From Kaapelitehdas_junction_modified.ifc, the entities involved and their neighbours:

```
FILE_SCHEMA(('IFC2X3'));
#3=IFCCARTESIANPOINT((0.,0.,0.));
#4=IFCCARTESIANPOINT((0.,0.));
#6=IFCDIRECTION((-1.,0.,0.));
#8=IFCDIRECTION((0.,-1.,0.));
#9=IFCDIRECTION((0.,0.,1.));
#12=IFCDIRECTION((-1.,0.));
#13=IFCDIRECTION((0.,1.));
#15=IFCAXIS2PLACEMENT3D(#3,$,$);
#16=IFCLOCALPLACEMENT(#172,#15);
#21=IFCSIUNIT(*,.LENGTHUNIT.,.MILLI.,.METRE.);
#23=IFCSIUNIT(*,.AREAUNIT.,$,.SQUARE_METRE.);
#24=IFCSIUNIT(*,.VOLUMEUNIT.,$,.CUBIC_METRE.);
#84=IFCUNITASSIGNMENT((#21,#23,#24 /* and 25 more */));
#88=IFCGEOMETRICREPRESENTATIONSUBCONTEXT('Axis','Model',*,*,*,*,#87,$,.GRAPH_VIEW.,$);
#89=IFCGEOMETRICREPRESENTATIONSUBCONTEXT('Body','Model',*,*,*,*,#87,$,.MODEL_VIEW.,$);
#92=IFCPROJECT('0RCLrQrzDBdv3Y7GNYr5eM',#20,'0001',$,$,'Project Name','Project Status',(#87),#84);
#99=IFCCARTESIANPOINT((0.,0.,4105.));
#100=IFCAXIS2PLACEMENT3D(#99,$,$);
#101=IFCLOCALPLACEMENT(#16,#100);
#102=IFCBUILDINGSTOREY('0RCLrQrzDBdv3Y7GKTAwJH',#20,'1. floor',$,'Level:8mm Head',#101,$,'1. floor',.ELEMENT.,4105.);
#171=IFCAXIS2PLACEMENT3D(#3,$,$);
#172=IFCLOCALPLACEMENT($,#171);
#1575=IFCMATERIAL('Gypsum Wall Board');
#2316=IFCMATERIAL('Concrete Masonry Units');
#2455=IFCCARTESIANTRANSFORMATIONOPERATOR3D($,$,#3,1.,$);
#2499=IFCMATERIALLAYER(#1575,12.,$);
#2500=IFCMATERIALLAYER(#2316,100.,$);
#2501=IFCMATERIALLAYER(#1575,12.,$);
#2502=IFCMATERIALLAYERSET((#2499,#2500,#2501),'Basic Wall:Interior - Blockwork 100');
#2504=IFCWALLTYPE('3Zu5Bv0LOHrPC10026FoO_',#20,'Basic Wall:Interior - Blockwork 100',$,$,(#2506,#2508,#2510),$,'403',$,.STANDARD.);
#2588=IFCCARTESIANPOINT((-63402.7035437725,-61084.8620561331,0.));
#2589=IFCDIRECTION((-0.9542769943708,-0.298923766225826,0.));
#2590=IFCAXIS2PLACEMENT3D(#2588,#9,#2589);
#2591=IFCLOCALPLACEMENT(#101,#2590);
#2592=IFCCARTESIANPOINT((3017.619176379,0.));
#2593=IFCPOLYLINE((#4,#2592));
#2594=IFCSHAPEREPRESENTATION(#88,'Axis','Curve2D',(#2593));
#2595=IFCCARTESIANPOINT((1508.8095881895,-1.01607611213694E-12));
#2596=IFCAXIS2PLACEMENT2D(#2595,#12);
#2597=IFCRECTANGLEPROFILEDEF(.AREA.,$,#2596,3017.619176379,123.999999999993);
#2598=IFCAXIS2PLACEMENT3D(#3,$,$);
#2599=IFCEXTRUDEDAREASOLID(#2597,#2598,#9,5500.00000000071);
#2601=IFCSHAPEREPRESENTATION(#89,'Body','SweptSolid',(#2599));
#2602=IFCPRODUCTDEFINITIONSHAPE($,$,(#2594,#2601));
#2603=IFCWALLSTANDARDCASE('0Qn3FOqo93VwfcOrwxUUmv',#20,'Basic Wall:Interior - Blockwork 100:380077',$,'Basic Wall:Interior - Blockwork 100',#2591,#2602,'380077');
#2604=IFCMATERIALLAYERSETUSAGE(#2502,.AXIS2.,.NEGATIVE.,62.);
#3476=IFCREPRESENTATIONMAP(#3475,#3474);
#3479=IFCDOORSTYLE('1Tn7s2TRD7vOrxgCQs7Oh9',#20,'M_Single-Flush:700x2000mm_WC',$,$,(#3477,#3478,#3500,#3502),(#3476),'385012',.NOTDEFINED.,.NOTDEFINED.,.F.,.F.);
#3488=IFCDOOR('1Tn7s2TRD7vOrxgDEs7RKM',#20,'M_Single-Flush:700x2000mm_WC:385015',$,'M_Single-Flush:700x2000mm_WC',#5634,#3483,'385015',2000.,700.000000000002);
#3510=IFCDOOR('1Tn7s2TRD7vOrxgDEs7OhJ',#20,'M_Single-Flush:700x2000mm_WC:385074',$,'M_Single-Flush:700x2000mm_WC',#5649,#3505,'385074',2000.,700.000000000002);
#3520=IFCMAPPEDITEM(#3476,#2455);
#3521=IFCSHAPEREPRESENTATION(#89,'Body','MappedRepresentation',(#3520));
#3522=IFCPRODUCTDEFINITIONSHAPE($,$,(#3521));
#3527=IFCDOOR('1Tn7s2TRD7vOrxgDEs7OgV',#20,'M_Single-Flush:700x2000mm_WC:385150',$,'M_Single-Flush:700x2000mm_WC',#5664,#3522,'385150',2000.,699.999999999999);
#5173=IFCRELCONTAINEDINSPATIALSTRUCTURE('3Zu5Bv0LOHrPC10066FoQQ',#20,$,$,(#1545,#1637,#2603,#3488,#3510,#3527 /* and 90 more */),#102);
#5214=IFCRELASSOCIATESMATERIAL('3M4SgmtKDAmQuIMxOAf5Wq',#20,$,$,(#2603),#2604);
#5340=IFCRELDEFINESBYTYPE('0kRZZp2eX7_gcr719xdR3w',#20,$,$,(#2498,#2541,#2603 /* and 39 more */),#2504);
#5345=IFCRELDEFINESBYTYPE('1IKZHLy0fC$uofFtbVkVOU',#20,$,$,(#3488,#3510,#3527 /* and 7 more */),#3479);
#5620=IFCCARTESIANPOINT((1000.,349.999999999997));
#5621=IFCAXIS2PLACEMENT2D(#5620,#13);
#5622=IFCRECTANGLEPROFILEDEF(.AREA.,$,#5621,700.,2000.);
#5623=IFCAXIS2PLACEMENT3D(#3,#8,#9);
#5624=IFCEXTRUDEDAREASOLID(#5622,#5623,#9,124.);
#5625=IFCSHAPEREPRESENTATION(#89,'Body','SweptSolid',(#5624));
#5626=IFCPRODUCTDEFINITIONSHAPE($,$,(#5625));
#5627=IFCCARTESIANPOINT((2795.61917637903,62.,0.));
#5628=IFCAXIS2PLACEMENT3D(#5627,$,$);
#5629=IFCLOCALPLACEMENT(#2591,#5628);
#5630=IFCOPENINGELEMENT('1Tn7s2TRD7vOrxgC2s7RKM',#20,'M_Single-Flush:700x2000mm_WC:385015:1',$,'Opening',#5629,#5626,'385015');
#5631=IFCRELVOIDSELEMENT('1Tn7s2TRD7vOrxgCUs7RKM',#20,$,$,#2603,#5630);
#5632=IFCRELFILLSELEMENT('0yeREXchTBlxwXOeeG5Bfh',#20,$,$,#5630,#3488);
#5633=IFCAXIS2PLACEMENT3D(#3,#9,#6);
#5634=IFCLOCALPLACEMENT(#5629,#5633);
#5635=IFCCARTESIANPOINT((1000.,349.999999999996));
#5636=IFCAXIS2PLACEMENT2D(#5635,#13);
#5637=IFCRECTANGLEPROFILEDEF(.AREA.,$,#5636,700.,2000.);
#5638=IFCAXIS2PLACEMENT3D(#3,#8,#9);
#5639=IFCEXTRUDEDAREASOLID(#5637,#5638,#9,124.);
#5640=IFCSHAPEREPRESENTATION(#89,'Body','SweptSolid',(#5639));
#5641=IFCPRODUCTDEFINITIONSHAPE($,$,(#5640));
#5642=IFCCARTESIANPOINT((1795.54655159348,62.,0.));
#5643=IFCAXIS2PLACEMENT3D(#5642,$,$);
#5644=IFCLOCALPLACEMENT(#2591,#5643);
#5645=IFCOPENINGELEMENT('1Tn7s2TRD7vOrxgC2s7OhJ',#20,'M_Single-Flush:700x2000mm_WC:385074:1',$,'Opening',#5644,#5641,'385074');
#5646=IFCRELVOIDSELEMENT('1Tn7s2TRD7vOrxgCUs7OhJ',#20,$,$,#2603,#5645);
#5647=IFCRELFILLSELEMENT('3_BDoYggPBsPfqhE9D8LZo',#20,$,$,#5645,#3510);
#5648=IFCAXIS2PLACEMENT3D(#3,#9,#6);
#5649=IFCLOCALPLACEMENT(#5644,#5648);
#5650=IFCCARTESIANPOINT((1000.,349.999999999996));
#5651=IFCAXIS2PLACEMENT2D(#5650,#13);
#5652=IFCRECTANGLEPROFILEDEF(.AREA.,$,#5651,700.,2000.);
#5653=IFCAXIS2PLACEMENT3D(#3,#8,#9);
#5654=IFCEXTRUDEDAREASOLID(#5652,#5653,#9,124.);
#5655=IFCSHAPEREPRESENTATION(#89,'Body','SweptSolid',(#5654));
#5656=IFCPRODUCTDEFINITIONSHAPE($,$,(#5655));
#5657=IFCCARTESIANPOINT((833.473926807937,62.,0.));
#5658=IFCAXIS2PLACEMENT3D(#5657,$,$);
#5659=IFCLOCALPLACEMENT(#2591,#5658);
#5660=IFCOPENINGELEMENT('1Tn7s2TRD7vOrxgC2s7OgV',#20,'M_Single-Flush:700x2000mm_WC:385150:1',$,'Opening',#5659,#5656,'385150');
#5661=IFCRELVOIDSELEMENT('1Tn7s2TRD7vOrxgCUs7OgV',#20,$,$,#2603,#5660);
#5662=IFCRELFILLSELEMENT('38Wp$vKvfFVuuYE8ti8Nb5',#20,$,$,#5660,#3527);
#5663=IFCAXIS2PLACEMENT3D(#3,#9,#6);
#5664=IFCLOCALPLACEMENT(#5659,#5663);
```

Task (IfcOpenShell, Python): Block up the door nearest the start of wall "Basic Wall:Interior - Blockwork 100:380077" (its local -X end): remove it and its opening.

```python
import ifcopenshell
import ifcopenshell.api.feature
import ifcopenshell.api.root
import ifcopenshell.geom
import ifcopenshell.util.shape

model = ifcopenshell.open("Kaapelitehdas_junction_modified.ifc")
settings = ifcopenshell.geom.settings()


def volume(element):
    """Net volume in cubic metres, openings subtracted."""
    shape = ifcopenshell.geom.create_shape(settings, element)
    return ifcopenshell.util.shape.get_volume(shape.geometry)


door = model.by_guid("1Tn7s2TRD7vOrxgDEs7OgV")
opening = door.FillsVoids[0].RelatingOpeningElement
wall = opening.VoidsElements[0].RelatingBuildingElement
before = volume(wall)

ifcopenshell.api.root.remove_product(model, product=door)
ifcopenshell.api.feature.remove_feature(model, feature=opening)

after = volume(wall)

print(f"wall volume {before:.3f} -> {after:.3f} m3")

model.write("Kaapelitehdas_junction_modified_v2.ifc")
```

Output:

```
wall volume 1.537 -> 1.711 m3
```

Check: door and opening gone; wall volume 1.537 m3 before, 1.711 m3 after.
